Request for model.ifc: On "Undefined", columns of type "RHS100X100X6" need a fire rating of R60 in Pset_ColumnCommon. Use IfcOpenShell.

First a look at what the model holds.

```python
import ifcopenshell
import ifcopenshell.util.element

model = ifcopenshell.open("model.ifc")
print(model.schema)
storey = next(s for s in model.by_type("IfcBuildingStorey") if s.Name == "Undefined")
columns = [e for e in ifcopenshell.util.element.get_decomposition(storey) if e.is_a("IfcColumn")]
seen = {}
for e in columns:
    element_type = ifcopenshell.util.element.get_type(e)
    key = (element_type.Name if element_type != e and element_type else None, ifcopenshell.util.element.get_pset(e, "Pset_ColumnCommon", "FireRating"))
    seen[key] = seen.get(key, 0) + 1
for (name, value), count in sorted(seen.items(), key=str):
    print(count, "x", name, "|", value)
```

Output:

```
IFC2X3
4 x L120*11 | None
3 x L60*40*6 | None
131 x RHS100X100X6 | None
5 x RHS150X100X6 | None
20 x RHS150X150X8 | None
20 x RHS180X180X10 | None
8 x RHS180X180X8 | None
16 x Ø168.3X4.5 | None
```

```python
import ifcopenshell
import ifcopenshell.api.pset
import ifcopenshell.util.element

model = ifcopenshell.open("model.ifc")

storey = next(s for s in model.by_type("IfcBuildingStorey") if s.Name == "Undefined")
columns = [e for e in ifcopenshell.util.element.get_decomposition(storey) if e.is_a("IfcColumn")]

count = 0
for e in columns:
    element_type = ifcopenshell.util.element.get_type(e)
    if element_type in (None, e) or element_type.Name != "RHS100X100X6":
        continue
    found = ifcopenshell.util.element.get_pset(e, "Pset_ColumnCommon", should_inherit=False)
    if found:
        pset = model.by_id(found["id"])
        if len(ifcopenshell.util.element.get_elements_by_pset(pset)) > 1:
            pset = ifcopenshell.api.pset.unshare_pset(model, products=[e], pset=pset)[0]
    else:
        pset = ifcopenshell.api.pset.add_pset(model, product=e, name="Pset_ColumnCommon")
    ifcopenshell.api.pset.edit_pset(model, pset=pset, properties={"FireRating": "R60"})
    count += 1

print(count, "columns updated")

model.write("model_updated.ifc")
```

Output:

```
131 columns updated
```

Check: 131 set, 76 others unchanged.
